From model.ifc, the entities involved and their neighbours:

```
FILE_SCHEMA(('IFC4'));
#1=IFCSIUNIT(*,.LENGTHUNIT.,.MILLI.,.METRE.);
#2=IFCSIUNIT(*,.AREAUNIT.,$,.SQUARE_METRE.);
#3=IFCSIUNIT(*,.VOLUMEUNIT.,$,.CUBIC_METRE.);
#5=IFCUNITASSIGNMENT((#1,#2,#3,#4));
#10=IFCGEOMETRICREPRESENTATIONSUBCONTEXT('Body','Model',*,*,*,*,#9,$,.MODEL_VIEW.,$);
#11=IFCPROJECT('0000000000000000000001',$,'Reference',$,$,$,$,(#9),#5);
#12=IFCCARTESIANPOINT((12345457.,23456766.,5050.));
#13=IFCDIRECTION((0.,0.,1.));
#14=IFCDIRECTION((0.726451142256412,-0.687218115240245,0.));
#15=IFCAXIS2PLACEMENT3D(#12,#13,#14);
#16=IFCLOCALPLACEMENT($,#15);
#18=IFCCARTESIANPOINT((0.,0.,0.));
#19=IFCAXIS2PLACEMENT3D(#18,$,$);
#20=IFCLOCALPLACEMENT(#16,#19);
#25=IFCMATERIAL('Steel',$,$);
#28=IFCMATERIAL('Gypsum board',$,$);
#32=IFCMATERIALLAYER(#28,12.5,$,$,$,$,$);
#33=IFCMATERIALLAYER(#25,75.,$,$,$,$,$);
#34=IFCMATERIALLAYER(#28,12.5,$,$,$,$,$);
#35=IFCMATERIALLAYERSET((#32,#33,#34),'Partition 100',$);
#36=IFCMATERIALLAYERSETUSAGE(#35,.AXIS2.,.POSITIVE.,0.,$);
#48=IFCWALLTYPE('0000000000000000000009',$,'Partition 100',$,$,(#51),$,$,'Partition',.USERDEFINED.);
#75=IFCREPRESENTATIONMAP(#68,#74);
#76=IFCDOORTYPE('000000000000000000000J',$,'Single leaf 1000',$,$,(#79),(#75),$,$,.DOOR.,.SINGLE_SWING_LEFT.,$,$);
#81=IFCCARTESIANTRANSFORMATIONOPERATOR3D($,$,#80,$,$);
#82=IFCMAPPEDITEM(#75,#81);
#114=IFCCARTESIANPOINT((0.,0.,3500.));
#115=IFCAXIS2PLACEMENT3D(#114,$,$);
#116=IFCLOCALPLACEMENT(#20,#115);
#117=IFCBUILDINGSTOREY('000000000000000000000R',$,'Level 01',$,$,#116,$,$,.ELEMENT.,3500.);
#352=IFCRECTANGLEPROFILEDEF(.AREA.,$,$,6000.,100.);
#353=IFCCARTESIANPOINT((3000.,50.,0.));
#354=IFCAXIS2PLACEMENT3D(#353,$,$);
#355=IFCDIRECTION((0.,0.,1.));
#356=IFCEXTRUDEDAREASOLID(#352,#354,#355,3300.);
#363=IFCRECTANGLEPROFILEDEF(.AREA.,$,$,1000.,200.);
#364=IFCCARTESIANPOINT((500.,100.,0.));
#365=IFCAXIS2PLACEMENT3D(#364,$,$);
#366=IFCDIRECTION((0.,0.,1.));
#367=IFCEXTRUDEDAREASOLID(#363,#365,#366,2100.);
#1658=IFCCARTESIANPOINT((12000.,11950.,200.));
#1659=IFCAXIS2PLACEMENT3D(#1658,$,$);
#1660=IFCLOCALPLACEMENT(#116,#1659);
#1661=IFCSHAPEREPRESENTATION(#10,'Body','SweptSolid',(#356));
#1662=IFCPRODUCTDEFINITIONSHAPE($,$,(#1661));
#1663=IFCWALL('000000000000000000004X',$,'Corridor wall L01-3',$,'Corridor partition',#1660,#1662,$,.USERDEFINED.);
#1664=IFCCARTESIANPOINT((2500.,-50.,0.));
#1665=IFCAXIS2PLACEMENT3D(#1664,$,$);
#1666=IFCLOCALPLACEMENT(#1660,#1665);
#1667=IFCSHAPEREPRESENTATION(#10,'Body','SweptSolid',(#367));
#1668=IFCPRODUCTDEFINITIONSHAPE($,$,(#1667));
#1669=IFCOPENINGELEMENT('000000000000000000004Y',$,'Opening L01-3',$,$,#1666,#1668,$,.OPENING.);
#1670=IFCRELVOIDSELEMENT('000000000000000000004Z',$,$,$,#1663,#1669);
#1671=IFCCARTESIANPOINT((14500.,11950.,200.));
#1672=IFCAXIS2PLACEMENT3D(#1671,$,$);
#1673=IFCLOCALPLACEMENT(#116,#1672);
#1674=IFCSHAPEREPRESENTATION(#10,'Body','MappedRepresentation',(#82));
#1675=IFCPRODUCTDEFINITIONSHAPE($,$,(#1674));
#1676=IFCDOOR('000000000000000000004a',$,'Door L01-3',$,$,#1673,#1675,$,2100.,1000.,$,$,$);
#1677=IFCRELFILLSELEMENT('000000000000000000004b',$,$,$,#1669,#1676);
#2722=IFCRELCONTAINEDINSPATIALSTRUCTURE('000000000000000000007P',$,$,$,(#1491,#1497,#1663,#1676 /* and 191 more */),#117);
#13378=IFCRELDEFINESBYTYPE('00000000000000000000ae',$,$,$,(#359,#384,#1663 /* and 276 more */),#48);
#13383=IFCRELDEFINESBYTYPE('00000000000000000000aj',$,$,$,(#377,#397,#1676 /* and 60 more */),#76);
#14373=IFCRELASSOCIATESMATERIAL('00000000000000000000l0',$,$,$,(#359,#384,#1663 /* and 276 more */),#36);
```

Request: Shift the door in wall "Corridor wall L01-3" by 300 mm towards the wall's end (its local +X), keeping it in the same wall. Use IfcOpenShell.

```python
import ifcopenshell
import ifcopenshell.api.geometry
import ifcopenshell.util.placement
import ifcopenshell.util.unit

model = ifcopenshell.open("model.ifc")
unit_scale = ifcopenshell.util.unit.calculate_unit_scale(model)

door = model.by_guid("000000000000000000004a")
opening = door.FillsVoids[0].RelatingOpeningElement
wall = opening.VoidsElements[0].RelatingBuildingElement

wall_matrix = ifcopenshell.util.placement.get_local_placement(wall.ObjectPlacement)
shift = wall_matrix[:3, 0] * 0.3 / unit_scale
before = ifcopenshell.util.placement.get_local_placement(door.ObjectPlacement)[:3, 3].copy()

# The door is not placed relative to its opening, so move both.
for product in (opening, door):
    matrix = ifcopenshell.util.placement.get_local_placement(product.ObjectPlacement)
    matrix[:3, 3] += shift
    ifcopenshell.api.geometry.edit_object_placement(model, product=product, matrix=matrix, is_si=False)

after = ifcopenshell.util.placement.get_local_placement(door.ObjectPlacement)[:3, 3]
print("door moved by", (after - before).round(3) + 0.0)

model.write("model_rev.ifc")
```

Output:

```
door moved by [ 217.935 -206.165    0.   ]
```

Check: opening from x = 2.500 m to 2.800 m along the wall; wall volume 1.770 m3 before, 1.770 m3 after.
